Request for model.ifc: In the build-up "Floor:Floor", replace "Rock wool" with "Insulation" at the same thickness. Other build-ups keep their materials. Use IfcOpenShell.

First a look at what the model holds.

```python
import ifcopenshell
import ifcopenshell.util.element

model = ifcopenshell.open("model.ifc")
print(model.schema)
for layer_set in model.by_type("IfcMaterialLayerSet"):
    if layer_set.LayerSetName == "Floor:Floor":
        for layer in layer_set.MaterialLayers:
            print(layer.id(), layer.Material and layer.Material.Name, layer.LayerThickness, sep=" | ")
        print(len(ifcopenshell.util.element.get_elements_by_material(model, layer_set)), "elements and types use it")
print(sorted(m.Name for m in model.by_type("IfcMaterial") if m.Name)[:60])
```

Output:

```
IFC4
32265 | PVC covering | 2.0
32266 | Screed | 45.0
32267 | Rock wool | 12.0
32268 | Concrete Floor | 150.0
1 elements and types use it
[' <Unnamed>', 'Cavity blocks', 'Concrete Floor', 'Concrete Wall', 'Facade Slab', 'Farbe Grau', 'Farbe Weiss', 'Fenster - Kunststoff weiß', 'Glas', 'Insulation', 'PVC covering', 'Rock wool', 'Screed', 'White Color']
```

```python
import ifcopenshell
import ifcopenshell.api.material

model = ifcopenshell.open("model.ifc")

layer_set = next(s for s in model.by_type("IfcMaterialLayerSet") if s.LayerSetName == "Floor:Floor")
layer = next(l for l in layer_set.MaterialLayers if l.Material and l.Material.Name == "Rock wool")
material = next(m for m in model.by_type("IfcMaterial") if m.Name == "Insulation")

# Point this one layer at the other material; renaming the old one would change it everywhere.
ifcopenshell.api.material.edit_layer(model, layer=layer, attributes={}, material=material)

print([l.Material.Name if l.Material else None for l in layer_set.MaterialLayers])

model.write("model_rev.ifc")
```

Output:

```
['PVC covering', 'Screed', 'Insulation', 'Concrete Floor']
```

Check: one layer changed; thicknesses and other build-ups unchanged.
